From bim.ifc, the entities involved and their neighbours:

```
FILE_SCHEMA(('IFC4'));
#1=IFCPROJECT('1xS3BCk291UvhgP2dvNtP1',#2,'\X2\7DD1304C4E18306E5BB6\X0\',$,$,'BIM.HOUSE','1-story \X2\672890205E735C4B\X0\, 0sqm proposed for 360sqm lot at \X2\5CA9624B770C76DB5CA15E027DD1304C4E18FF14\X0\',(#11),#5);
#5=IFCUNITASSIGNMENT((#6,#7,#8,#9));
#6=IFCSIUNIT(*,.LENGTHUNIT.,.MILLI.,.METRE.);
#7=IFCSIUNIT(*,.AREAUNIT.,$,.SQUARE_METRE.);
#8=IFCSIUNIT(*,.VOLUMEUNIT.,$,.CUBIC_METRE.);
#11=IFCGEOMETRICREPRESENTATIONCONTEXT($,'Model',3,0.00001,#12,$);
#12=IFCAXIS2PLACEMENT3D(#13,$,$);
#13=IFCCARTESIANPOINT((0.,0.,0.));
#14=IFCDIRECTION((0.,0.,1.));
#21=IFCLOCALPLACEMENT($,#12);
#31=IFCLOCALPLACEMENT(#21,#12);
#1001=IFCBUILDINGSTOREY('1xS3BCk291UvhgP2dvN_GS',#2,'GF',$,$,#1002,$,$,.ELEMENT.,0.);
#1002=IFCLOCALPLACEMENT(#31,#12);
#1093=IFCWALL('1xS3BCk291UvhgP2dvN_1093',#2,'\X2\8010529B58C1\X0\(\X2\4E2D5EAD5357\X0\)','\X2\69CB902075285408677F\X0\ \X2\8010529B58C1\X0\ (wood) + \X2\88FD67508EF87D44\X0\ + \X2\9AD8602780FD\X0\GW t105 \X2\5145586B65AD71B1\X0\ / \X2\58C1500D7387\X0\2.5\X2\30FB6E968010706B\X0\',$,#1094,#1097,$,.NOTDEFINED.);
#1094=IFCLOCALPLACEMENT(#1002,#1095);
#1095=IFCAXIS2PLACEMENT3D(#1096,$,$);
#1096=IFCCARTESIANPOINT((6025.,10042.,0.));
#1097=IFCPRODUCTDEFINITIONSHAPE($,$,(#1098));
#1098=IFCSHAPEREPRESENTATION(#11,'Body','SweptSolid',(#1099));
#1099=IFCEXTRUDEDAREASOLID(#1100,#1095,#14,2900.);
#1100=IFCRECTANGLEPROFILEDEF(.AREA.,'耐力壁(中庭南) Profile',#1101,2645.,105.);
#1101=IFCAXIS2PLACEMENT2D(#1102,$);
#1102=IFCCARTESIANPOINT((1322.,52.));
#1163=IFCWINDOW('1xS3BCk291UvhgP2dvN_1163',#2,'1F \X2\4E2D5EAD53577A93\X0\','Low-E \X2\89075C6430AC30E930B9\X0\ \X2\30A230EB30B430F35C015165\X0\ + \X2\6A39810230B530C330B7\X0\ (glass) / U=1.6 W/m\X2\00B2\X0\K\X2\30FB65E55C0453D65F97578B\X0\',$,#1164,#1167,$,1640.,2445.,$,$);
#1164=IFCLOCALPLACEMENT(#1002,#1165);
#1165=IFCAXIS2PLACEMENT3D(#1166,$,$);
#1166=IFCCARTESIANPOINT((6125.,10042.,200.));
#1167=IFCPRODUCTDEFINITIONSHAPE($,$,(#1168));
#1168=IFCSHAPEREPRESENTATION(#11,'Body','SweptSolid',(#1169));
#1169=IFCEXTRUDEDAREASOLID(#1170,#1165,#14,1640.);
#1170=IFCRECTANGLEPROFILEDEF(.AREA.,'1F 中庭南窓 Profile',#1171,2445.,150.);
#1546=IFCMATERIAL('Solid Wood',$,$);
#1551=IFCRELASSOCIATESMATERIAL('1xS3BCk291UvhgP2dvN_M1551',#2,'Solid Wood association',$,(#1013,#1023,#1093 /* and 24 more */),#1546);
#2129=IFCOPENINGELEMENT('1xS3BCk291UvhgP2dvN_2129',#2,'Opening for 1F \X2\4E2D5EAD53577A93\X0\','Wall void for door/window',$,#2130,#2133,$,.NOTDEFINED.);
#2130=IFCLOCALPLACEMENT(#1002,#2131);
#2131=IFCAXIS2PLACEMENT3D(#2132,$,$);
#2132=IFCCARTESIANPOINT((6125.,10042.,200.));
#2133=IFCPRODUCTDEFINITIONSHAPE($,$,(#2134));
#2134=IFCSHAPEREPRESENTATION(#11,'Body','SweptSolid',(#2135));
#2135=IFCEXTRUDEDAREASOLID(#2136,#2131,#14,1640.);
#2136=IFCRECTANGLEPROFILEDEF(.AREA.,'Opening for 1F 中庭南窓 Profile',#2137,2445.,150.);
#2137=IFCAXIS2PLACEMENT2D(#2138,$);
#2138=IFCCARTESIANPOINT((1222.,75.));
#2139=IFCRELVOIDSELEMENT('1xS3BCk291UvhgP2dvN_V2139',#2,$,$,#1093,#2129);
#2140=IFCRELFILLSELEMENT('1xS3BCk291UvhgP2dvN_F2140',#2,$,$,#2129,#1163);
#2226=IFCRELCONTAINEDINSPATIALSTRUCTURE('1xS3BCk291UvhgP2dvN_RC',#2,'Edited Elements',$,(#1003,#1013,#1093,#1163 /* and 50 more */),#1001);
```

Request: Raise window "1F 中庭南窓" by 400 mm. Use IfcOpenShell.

```python
import numpy as np
import ifcopenshell
import ifcopenshell.api.geometry
import ifcopenshell.util.placement
import ifcopenshell.util.unit

model = ifcopenshell.open("bim.ifc")
unit_scale = ifcopenshell.util.unit.calculate_unit_scale(model)

window = model.by_guid("1xS3BCk291UvhgP2dvN_1163")
opening = window.FillsVoids[0].RelatingOpeningElement
dz = 400.0

shift = np.array([0.0, 0.0, dz])
# The window is not placed relative to its opening, so move both.
for product in (opening, window):
    matrix = ifcopenshell.util.placement.get_local_placement(product.ObjectPlacement)
    matrix[:3, 3] += shift
    ifcopenshell.api.geometry.edit_object_placement(model, product=product, matrix=matrix, is_si=False)

print(f"moved by {dz * unit_scale:+.3f} m")

model.write("bim_updated.ifc")
```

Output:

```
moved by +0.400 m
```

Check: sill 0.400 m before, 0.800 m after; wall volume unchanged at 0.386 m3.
